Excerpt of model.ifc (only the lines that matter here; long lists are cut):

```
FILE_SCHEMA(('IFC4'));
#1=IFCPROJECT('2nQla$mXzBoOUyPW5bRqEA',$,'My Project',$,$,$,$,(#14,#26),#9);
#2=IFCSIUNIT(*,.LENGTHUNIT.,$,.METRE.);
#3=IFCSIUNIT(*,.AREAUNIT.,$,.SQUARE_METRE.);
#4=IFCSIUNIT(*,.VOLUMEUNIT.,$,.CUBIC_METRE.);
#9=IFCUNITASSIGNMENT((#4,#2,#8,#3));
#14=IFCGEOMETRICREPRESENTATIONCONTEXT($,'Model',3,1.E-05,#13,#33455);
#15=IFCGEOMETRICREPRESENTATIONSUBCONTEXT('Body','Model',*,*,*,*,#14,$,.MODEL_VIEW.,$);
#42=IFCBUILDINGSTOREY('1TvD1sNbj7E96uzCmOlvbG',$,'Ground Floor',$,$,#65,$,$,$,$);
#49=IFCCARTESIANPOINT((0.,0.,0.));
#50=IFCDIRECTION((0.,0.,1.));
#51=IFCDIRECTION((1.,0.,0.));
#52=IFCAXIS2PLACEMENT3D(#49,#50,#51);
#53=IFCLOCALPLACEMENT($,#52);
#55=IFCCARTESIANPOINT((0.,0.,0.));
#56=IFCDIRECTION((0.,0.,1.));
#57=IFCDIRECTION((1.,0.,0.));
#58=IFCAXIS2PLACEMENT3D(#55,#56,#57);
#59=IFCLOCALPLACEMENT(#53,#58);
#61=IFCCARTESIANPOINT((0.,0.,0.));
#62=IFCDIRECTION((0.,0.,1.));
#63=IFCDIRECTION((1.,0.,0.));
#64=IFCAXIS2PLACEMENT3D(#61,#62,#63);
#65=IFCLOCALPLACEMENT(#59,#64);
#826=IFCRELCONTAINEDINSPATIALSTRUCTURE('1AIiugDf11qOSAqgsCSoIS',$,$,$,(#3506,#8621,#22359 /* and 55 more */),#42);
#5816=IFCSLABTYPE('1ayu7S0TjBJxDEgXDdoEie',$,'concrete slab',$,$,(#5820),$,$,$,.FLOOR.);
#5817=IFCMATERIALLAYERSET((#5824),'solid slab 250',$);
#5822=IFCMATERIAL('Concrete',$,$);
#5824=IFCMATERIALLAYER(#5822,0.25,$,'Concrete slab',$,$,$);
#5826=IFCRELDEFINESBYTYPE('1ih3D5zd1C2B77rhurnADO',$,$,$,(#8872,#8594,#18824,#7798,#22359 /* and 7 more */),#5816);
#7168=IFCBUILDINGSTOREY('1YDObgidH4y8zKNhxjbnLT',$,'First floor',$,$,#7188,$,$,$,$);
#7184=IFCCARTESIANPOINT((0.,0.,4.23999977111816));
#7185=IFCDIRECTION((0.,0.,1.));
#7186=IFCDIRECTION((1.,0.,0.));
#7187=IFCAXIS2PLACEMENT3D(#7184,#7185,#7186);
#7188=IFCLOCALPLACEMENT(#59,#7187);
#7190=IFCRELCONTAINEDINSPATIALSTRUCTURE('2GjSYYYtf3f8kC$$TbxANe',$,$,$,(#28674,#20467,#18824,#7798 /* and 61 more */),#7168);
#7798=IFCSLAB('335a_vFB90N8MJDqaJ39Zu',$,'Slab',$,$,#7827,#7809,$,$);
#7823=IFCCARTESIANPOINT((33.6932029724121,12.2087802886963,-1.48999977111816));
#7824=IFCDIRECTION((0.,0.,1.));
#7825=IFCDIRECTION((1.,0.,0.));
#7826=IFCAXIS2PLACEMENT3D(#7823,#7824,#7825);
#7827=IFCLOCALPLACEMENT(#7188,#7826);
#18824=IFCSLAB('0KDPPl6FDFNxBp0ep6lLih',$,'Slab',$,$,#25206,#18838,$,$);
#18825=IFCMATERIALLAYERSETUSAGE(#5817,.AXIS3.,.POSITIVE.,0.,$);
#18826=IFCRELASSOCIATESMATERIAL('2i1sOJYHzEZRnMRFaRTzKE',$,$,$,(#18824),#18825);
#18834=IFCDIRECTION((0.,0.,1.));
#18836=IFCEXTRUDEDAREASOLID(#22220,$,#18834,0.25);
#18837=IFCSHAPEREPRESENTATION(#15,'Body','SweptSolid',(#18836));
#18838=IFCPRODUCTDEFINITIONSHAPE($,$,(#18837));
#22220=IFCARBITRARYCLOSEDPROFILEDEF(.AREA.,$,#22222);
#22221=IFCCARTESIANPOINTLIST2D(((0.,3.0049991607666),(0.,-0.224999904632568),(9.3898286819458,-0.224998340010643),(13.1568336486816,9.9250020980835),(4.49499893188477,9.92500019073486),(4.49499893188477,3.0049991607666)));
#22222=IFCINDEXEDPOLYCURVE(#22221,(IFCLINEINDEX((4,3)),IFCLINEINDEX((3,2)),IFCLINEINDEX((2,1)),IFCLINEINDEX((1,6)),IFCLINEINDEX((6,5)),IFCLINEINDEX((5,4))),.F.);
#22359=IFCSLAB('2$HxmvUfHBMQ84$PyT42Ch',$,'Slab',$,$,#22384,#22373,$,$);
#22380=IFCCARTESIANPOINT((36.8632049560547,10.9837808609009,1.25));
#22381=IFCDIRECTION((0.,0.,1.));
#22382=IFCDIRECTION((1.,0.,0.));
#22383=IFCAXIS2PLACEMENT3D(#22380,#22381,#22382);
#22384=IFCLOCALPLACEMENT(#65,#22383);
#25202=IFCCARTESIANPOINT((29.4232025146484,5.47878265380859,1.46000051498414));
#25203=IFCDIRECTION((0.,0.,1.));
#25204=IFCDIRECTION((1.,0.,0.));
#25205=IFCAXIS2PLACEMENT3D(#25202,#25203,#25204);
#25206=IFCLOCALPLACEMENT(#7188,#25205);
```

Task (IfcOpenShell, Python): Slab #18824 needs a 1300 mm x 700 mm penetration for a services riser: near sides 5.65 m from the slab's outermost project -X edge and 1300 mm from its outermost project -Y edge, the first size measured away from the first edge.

```python
import numpy as np
import ifcopenshell
import ifcopenshell.api.feature
import ifcopenshell.api.geometry
import ifcopenshell.api.root
import ifcopenshell.geom
import ifcopenshell.util.placement
import ifcopenshell.util.representation
import ifcopenshell.util.shape
import ifcopenshell.util.unit

model = ifcopenshell.open("model.ifc")
unit_scale = ifcopenshell.util.unit.calculate_unit_scale(model)
settings = ifcopenshell.geom.settings()


def volume(element):
    """Net volume in cubic metres, openings subtracted."""
    shape = ifcopenshell.geom.create_shape(settings, element)
    return ifcopenshell.util.shape.get_volume(shape.geometry)


slab = model.by_guid("0KDPPl6FDFNxBp0ep6lLih")
before = volume(slab)

# Extent in the slab's own axes, in metres. The edges named are its -X and -Y sides.
slab_shape = ifcopenshell.geom.create_shape(settings, slab)
vertices = ifcopenshell.util.shape.get_vertices(slab_shape.geometry)
x_min, y_min, bottom = vertices.min(axis=0)
top = vertices[:, 2].max()

opening = ifcopenshell.api.root.create_entity(model, ifc_class="IfcOpeningElement", name="Services riser opening", predefined_type="OPENING")
context = ifcopenshell.util.representation.get_context(model, "Model", "Body", "MODEL_VIEW")
width, depth = 1.3, 0.7
outline = [(0.0, 0.0), (width, 0.0), (width, depth), (0.0, depth), (0.0, 0.0)]
# Overshoot both faces by 50 mm so the cut is clean.
shape = ifcopenshell.api.geometry.add_slab_representation(
    model, context=context, depth=top - bottom + 0.1, polyline=outline
)
ifcopenshell.api.geometry.assign_representation(model, product=opening, representation=shape)

matrix = ifcopenshell.util.placement.get_local_placement(slab.ObjectPlacement)
matrix[:, 3] = matrix @ np.append(np.array([x_min + 5.65, y_min + 1.3, bottom - 0.05]) / unit_scale, 1.0)
ifcopenshell.api.geometry.edit_object_placement(model, product=opening, matrix=matrix, is_si=False)
ifcopenshell.api.feature.add_feature(model, feature=opening, element=slab)

after = volume(slab)

print(f"slab volume {before:.3f} -> {after:.3f} m3")

model.write("model_rev.ifc")
```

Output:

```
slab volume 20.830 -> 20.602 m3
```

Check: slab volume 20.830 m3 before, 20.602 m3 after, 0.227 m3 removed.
